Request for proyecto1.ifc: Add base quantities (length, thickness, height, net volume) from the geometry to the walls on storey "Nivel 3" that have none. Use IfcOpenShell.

First a look at what the model holds.

```python
import ifcopenshell
import ifcopenshell.util.element
import ifcopenshell.util.unit

model = ifcopenshell.open("proyecto1.ifc")
print(model.schema)
for unit_type in ("LENGTHUNIT", "AREAUNIT", "VOLUMEUNIT"):
    print(unit_type, ifcopenshell.util.unit.calculate_unit_scale(model, unit_type))
storey = next(s for s in model.by_type("IfcBuildingStorey") if s.Name == "Nivel 3")
walls = [e for e in ifcopenshell.util.element.get_decomposition(storey) if e.is_a("IfcWall")]
for e in sorted(walls, key=lambda e: e.id()):
    print(e.id(), e.is_a(), e.Name, list(ifcopenshell.util.element.get_psets(e, qtos_only=True)), sep=" | ")
```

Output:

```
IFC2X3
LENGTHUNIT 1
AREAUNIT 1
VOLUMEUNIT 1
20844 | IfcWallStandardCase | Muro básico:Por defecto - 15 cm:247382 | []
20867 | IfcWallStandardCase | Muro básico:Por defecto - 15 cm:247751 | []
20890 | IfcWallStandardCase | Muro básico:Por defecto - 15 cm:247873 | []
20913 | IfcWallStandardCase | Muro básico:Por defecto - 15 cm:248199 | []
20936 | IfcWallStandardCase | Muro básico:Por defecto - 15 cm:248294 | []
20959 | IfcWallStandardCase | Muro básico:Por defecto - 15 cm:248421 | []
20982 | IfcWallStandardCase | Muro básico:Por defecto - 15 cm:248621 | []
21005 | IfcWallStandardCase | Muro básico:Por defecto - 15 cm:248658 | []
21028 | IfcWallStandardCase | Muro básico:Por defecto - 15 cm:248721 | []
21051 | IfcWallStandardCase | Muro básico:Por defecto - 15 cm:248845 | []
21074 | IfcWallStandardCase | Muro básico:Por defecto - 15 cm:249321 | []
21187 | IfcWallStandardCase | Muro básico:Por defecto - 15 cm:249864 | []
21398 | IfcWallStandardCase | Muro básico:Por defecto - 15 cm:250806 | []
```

```python
import ifcopenshell
import ifcopenshell.api.pset
import ifcopenshell.geom
import ifcopenshell.util.element
import ifcopenshell.util.shape
import ifcopenshell.util.unit

model = ifcopenshell.open("proyecto1.ifc")
unit_scale = ifcopenshell.util.unit.calculate_unit_scale(model)
volume_scale = ifcopenshell.util.unit.calculate_unit_scale(model, "VOLUMEUNIT")
settings = ifcopenshell.geom.settings()

storey = next(s for s in model.by_type("IfcBuildingStorey") if s.Name == "Nivel 3")
walls = [e for e in ifcopenshell.util.element.get_decomposition(storey) if e.is_a("IfcWall")]

for e in sorted(walls, key=lambda e: e.id()):
    if ifcopenshell.util.element.get_psets(e, qtos_only=True, should_inherit=False):
        continue
    # Geometry comes back in metres, in the element's own axes.
    shape = ifcopenshell.geom.create_shape(settings, e)
    values = {
        "Length": ifcopenshell.util.shape.get_x(shape.geometry) / unit_scale,
        "Width": ifcopenshell.util.shape.get_y(shape.geometry) / unit_scale,
        "Height": ifcopenshell.util.shape.get_z(shape.geometry) / unit_scale,
        "NetVolume": ifcopenshell.util.shape.get_volume(shape.geometry) / volume_scale,
    }
    qto = ifcopenshell.api.pset.add_qto(model, product=e, name="BaseQuantities")
    ifcopenshell.api.pset.edit_qto(model, qto=qto, properties=values)
    print(e.id(), {k: round(v, 3) for k, v in values.items()})

model.write("proyecto1_updated.ifc")
```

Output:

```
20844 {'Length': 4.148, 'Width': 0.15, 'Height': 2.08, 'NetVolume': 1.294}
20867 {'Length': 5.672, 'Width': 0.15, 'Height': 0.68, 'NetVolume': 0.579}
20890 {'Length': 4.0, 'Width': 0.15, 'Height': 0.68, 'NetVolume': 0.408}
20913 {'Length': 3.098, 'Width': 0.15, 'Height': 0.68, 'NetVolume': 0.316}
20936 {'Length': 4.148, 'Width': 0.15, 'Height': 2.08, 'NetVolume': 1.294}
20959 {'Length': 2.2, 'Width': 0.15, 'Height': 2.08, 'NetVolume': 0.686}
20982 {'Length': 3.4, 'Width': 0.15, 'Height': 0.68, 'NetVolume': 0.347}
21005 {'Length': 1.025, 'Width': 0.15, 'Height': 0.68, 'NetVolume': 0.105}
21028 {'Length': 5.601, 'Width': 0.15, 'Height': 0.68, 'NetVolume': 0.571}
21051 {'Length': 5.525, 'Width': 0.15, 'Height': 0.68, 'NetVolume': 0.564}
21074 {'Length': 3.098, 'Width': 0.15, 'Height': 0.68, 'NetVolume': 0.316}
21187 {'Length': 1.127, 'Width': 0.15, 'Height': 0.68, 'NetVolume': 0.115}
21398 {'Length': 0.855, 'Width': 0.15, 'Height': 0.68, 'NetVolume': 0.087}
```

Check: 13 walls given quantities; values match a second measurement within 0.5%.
